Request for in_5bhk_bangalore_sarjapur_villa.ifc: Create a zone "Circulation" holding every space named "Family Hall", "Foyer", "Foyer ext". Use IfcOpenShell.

First a look at what the model holds.

```python
import ifcopenshell

model = ifcopenshell.open("in_5bhk_bangalore_sarjapur_villa.ifc")
print(model.schema)
seen = {}
for space in model.by_type("IfcSpace"):
    seen[space.LongName] = seen.get(space.LongName, 0) + 1
for name, count in sorted(seen.items(), key=str):
    print(count, "x", name)
print("zones:", [z.Name for z in model.by_type("IfcZone")][:20])
```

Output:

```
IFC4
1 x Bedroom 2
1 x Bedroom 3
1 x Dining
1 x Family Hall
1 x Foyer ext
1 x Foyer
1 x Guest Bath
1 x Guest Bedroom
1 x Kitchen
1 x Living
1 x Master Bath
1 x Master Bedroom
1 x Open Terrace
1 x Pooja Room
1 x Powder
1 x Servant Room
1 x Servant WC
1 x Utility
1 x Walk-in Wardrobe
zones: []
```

```python
import ifcopenshell
import ifcopenshell.api.group
import ifcopenshell.api.root

model = ifcopenshell.open("in_5bhk_bangalore_sarjapur_villa.ifc")

names = {"Family Hall", "Foyer", "Foyer ext"}
spaces = [s for s in model.by_type("IfcSpace") if s.LongName in names]

zone = ifcopenshell.api.root.create_entity(model, ifc_class="IfcZone", name="Circulation")
ifcopenshell.api.group.assign_group(model, products=spaces, group=zone)
print(len(spaces), "spaces in", zone.Name)

model.write("in_5bhk_bangalore_sarjapur_villa-out.ifc")
```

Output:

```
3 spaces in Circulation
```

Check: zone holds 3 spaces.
